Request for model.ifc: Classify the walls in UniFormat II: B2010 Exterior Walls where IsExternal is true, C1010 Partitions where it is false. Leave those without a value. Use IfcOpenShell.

First a look at what the model holds.

```python
import ifcopenshell
import ifcopenshell.util.element

model = ifcopenshell.open("model.ifc")
print(model.schema)
print("classifications:", [c.Name for c in model.by_type("IfcClassification")])
values = [ifcopenshell.util.element.get_pset(e, "Pset_WallCommon", "IsExternal") for e in model.by_type("IfcWall")]
for value in (True, False, None):
    print("IsExternal", value, values.count(value))
```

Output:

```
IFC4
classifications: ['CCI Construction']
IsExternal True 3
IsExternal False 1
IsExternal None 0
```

```python
import ifcopenshell
import ifcopenshell.api.classification
import ifcopenshell.util.element

model = ifcopenshell.open("model.ifc")

system = ifcopenshell.api.classification.add_classification(model, classification="UniFormat II")

walls = model.by_type("IfcWall")
external = {e: ifcopenshell.util.element.get_pset(e, "Pset_WallCommon", "IsExternal") for e in walls}
for flag, code, name in ((True, "B2010", "Exterior Walls"), (False, "C1010", "Partitions")):
    products = [e for e in walls if external[e] is flag]
    ifcopenshell.api.classification.add_reference(
        model, products=products, classification=system, identification=code, name=name
    )
    print(code, len(products))

model.write("model_edited.ifc")
```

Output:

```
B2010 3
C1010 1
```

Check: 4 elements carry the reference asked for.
